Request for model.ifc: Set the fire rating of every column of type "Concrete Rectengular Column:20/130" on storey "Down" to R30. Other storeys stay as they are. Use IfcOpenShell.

First a look at what the model holds.

```python
import ifcopenshell
import ifcopenshell.util.element

model = ifcopenshell.open("model.ifc")
print(model.schema)
storey = next(s for s in model.by_type("IfcBuildingStorey") if s.Name == "Down")
columns = [e for e in ifcopenshell.util.element.get_decomposition(storey) if e.is_a("IfcColumn")]
seen = {}
for e in columns:
    element_type = ifcopenshell.util.element.get_type(e)
    key = (element_type.Name if element_type != e and element_type else None, ifcopenshell.util.element.get_pset(e, "Pset_ColumnCommon", "FireRating"))
    seen[key] = seen.get(key, 0) + 1
for (name, value), count in sorted(seen.items(), key=str):
    print(count, "x", name, "|", value)
```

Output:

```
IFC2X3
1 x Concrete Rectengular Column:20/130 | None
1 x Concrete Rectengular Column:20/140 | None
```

```python
import ifcopenshell
import ifcopenshell.api.pset
import ifcopenshell.util.element

model = ifcopenshell.open("model.ifc")

storey = next(s for s in model.by_type("IfcBuildingStorey") if s.Name == "Down")
columns = [e for e in ifcopenshell.util.element.get_decomposition(storey) if e.is_a("IfcColumn")]

count = 0
for e in columns:
    element_type = ifcopenshell.util.element.get_type(e)
    if element_type in (None, e) or element_type.Name != "Concrete Rectengular Column:20/130":
        continue
    # add_pset returns the element's existing set when there is one.
    pset = ifcopenshell.api.pset.add_pset(model, product=e, name="Pset_ColumnCommon")
    ifcopenshell.api.pset.edit_pset(model, pset=pset, properties={"FireRating": "R30"})
    count += 1

print(count, "columns updated")

model.write("model_rev.ifc")
```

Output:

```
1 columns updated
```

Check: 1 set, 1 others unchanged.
